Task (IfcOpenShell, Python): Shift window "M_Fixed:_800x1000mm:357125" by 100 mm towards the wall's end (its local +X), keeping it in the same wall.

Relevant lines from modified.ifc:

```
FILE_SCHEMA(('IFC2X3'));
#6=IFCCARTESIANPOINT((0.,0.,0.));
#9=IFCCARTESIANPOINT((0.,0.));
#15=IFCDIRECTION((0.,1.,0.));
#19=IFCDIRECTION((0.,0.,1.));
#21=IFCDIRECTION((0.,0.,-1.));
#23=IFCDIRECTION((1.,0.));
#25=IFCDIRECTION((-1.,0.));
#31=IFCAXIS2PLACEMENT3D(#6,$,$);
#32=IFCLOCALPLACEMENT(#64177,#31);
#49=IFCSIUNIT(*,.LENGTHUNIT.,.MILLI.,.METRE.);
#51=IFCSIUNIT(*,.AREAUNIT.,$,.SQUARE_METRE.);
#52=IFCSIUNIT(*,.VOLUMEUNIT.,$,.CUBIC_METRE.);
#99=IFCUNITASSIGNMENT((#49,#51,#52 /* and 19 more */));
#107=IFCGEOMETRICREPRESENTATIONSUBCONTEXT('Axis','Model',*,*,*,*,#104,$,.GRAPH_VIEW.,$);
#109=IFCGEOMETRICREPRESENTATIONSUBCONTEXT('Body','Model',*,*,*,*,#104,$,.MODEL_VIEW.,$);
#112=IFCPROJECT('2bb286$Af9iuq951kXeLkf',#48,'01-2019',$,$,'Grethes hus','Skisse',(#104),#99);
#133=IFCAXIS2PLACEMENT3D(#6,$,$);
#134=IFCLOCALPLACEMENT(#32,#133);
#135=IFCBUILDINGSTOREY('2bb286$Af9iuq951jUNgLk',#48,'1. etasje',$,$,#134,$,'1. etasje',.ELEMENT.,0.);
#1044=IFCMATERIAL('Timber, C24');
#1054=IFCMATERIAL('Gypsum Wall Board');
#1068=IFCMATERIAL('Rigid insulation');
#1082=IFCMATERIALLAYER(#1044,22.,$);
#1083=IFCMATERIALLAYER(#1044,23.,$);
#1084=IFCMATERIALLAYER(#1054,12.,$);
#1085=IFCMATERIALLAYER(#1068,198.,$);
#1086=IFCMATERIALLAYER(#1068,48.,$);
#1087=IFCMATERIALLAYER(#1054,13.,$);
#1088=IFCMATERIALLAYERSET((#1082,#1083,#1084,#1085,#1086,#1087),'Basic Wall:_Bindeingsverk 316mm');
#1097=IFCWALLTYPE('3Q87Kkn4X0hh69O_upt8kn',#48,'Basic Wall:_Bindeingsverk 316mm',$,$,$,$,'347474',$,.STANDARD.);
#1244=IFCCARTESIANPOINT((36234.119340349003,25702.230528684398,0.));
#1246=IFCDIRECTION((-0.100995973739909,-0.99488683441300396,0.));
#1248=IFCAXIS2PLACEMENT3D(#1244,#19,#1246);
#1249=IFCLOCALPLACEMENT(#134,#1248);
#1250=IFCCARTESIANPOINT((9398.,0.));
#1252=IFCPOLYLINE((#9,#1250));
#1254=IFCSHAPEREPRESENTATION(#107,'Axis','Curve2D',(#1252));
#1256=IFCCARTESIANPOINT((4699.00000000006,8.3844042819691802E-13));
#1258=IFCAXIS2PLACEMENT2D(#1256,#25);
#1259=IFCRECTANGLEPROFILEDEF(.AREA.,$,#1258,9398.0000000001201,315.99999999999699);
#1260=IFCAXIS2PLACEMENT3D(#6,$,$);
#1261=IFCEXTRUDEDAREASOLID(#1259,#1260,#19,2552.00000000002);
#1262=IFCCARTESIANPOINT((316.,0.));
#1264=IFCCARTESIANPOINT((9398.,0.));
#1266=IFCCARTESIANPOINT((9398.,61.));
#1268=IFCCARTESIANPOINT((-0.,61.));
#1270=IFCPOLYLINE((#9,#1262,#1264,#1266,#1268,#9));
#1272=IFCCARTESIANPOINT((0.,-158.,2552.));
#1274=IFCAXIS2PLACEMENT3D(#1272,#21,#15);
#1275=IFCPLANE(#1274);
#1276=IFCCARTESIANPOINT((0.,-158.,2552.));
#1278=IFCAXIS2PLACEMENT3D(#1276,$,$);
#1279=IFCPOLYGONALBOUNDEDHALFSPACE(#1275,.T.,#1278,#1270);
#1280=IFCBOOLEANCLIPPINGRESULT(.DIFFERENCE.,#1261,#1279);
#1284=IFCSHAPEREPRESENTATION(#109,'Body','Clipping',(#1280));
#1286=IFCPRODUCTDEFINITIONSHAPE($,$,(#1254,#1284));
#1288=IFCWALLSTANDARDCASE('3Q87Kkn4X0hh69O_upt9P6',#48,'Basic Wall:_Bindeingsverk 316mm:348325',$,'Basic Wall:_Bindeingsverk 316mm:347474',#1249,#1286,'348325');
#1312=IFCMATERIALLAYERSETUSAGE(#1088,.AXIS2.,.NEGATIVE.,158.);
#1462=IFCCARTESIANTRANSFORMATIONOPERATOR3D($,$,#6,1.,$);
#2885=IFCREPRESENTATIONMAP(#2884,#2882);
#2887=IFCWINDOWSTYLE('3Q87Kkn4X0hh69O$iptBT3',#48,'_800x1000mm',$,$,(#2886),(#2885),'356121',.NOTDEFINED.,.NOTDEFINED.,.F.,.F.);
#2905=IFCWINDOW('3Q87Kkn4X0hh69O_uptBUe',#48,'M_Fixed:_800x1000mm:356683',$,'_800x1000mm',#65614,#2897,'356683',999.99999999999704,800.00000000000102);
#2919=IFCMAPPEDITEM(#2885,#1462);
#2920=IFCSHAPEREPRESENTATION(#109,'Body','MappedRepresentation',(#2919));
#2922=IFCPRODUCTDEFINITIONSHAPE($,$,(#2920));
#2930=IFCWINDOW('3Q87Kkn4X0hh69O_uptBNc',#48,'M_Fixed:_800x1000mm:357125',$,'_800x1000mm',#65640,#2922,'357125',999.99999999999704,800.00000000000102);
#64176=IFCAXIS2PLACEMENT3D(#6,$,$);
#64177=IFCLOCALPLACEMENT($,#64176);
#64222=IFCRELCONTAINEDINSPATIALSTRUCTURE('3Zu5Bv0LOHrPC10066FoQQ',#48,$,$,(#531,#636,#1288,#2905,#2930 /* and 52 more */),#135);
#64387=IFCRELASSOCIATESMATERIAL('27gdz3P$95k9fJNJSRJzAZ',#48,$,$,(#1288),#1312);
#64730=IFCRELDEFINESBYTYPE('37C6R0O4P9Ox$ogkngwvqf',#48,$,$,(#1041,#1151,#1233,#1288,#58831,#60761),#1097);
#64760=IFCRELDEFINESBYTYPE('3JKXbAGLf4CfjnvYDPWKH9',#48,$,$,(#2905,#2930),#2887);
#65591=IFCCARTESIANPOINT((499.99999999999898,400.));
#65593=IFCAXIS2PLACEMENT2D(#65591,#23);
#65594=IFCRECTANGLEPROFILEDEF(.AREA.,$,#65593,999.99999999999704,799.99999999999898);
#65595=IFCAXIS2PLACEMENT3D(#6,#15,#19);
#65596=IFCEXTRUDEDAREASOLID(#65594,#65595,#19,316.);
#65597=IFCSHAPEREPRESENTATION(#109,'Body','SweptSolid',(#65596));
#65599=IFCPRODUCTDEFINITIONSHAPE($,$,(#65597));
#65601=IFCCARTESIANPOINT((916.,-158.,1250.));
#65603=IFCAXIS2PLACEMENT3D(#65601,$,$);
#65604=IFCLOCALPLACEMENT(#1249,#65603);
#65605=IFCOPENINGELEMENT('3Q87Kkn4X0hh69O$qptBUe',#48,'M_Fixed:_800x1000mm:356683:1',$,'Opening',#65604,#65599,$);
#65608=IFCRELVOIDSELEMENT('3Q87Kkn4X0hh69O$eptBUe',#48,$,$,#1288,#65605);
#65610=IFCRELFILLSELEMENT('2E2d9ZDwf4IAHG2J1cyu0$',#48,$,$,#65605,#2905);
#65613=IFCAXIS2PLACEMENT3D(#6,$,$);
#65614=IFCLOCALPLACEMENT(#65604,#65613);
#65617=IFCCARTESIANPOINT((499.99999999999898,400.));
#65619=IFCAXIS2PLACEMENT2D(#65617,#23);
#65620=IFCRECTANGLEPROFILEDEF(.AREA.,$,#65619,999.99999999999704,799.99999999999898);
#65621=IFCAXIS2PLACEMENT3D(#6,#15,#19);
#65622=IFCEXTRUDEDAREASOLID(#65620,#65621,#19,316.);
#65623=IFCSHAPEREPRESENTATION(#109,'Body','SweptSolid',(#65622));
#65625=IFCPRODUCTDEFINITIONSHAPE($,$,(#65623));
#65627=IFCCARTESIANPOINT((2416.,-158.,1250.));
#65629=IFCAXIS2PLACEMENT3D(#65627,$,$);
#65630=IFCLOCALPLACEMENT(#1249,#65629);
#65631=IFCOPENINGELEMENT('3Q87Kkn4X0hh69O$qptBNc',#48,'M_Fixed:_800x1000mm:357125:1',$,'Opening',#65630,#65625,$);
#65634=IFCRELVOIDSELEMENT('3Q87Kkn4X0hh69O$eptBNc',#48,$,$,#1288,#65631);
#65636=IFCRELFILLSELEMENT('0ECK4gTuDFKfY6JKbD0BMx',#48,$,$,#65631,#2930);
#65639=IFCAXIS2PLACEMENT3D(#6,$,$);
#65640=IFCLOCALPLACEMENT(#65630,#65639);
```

```python
import ifcopenshell
import ifcopenshell.api.geometry
import ifcopenshell.util.placement
import ifcopenshell.util.unit

model = ifcopenshell.open("modified.ifc")
unit_scale = ifcopenshell.util.unit.calculate_unit_scale(model)

window = model.by_guid("3Q87Kkn4X0hh69O_uptBNc")
opening = window.FillsVoids[0].RelatingOpeningElement
wall = opening.VoidsElements[0].RelatingBuildingElement

wall_matrix = ifcopenshell.util.placement.get_local_placement(wall.ObjectPlacement)
shift = wall_matrix[:3, 0] * 0.1 / unit_scale
before = ifcopenshell.util.placement.get_local_placement(window.ObjectPlacement)[:3, 3].copy()

# The window is placed relative to its opening, so it follows when the opening moves.
matrix = ifcopenshell.util.placement.get_local_placement(opening.ObjectPlacement)
matrix[:3, 3] += shift
ifcopenshell.api.geometry.edit_object_placement(
    model, product=opening, matrix=matrix, is_si=False, should_transform_children=True
)

after = ifcopenshell.util.placement.get_local_placement(window.ObjectPlacement)[:3, 3]
print("window moved by", (after - before).round(3) + 0.0)

model.write("modified-out.ifc")
```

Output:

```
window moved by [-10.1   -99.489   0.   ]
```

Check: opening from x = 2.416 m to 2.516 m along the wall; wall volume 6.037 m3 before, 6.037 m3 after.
